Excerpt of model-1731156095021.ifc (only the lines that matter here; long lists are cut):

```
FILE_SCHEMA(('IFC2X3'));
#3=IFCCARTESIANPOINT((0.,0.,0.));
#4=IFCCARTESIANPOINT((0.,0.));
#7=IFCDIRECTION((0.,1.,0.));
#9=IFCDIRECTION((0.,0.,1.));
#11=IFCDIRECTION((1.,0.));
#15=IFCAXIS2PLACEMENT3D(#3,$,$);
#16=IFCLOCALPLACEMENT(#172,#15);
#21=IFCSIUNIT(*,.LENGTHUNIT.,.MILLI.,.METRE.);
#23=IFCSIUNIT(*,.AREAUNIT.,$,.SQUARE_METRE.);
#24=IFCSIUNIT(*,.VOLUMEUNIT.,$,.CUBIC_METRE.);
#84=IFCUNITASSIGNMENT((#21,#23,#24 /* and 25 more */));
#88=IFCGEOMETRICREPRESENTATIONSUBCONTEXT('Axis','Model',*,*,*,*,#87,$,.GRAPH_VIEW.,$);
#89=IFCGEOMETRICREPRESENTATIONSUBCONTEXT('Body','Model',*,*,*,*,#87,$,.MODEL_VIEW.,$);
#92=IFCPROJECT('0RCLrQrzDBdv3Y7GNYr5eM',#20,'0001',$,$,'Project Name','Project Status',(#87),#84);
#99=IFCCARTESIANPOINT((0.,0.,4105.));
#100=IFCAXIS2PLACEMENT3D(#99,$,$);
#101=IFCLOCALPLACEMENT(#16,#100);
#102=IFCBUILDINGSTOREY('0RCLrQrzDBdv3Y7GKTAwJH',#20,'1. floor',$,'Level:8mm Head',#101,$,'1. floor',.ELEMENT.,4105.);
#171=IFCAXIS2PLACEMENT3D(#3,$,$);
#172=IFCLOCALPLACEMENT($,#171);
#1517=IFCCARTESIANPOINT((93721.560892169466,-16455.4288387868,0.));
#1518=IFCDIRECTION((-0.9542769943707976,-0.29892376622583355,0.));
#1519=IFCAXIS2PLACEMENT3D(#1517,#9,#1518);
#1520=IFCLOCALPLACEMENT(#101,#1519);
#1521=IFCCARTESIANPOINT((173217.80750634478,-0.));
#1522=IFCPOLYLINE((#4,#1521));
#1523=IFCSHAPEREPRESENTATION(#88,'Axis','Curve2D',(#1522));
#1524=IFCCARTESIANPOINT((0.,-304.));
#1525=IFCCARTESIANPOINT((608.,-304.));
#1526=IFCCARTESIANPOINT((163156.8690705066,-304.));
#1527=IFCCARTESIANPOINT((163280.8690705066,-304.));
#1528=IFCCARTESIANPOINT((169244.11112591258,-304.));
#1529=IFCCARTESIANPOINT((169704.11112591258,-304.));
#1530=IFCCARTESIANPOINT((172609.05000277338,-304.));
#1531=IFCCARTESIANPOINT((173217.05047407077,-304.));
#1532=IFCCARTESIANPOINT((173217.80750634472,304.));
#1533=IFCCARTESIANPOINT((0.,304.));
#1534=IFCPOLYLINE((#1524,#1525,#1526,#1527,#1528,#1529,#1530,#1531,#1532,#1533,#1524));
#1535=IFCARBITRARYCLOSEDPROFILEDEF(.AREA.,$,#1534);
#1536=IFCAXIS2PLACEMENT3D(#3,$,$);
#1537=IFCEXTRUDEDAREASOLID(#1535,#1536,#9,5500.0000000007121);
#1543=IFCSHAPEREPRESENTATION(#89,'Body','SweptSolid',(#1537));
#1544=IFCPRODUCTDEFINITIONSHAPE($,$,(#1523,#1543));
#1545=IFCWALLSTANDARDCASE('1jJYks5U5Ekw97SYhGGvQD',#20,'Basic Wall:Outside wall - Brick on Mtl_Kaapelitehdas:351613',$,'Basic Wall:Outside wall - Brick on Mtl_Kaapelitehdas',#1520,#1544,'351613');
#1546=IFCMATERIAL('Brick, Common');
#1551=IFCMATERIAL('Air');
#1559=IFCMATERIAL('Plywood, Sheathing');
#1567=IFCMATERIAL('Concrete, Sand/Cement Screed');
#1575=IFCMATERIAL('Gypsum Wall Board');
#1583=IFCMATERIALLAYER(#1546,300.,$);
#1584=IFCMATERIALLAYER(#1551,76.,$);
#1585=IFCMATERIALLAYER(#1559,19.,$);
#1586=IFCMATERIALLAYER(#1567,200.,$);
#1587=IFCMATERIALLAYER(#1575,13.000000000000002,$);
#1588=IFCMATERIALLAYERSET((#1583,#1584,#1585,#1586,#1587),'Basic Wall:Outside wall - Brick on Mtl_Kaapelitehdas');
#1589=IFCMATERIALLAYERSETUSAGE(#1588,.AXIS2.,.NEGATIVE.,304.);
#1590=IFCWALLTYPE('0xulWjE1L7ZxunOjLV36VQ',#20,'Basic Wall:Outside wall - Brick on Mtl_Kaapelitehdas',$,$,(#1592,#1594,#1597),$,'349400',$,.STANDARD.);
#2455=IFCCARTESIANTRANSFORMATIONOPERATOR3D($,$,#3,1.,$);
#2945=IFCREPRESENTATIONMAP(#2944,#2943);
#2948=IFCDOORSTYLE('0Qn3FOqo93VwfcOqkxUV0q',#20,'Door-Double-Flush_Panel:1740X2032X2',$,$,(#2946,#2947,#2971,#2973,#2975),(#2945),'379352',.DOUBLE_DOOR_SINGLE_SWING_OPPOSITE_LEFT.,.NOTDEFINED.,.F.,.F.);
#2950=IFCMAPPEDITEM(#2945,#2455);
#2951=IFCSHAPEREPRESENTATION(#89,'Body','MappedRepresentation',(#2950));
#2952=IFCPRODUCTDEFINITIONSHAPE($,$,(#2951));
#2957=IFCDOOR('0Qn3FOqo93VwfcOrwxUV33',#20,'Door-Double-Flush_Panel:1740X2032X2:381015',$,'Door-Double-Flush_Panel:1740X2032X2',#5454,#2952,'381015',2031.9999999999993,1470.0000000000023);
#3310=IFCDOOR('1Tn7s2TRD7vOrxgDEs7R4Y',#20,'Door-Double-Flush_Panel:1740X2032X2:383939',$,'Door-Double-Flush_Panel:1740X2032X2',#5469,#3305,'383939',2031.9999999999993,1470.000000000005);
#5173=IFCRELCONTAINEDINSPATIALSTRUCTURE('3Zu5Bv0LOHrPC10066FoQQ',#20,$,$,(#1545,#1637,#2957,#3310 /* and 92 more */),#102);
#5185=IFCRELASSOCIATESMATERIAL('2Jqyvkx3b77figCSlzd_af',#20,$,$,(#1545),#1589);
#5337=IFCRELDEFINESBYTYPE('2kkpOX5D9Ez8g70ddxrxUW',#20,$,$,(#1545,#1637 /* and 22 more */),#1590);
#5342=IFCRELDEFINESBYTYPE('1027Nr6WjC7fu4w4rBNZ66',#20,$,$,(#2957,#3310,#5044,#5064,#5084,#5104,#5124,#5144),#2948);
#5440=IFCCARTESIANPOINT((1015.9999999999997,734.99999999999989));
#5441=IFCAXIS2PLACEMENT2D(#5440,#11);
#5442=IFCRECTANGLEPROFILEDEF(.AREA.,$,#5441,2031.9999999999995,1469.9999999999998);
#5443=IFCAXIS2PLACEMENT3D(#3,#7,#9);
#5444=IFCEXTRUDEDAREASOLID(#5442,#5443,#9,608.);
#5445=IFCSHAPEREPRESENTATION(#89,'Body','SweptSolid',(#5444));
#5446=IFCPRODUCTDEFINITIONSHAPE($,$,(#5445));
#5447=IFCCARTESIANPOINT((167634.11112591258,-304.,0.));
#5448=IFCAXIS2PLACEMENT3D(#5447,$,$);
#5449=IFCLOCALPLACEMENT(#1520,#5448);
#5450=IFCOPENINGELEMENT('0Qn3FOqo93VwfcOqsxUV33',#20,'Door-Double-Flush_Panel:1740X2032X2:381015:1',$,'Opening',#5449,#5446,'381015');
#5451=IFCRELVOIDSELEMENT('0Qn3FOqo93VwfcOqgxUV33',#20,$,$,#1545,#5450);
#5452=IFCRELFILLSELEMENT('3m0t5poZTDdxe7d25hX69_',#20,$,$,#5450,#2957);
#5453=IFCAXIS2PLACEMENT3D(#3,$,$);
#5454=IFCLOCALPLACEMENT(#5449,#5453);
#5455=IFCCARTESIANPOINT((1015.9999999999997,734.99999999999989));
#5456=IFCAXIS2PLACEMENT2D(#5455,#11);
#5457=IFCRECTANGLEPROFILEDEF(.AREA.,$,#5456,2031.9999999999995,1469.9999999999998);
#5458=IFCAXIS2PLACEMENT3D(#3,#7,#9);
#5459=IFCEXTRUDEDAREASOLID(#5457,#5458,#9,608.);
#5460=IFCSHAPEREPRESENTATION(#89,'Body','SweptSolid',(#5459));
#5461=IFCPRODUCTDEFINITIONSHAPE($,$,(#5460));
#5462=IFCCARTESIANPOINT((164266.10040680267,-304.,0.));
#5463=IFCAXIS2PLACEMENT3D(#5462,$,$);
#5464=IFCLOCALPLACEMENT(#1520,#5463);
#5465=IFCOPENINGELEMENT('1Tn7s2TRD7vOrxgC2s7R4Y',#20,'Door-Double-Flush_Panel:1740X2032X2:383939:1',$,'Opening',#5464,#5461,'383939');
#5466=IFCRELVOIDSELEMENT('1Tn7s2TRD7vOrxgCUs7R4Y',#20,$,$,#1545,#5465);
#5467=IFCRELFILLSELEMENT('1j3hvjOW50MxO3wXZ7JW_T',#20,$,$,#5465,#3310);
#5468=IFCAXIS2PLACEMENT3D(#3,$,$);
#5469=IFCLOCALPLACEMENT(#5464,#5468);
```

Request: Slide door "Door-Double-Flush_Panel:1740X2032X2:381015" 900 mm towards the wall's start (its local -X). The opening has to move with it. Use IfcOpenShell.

```python
import ifcopenshell
import ifcopenshell.api.geometry
import ifcopenshell.util.placement
import ifcopenshell.util.unit

model = ifcopenshell.open("model-1731156095021.ifc")
unit_scale = ifcopenshell.util.unit.calculate_unit_scale(model)

door = model.by_guid("0Qn3FOqo93VwfcOrwxUV33")
opening = door.FillsVoids[0].RelatingOpeningElement
wall = opening.VoidsElements[0].RelatingBuildingElement

wall_matrix = ifcopenshell.util.placement.get_local_placement(wall.ObjectPlacement)
shift = wall_matrix[:3, 0] * -0.9 / unit_scale
before = ifcopenshell.util.placement.get_local_placement(door.ObjectPlacement)[:3, 3].copy()

# The door is placed relative to its opening, so it follows when the opening moves.
matrix = ifcopenshell.util.placement.get_local_placement(opening.ObjectPlacement)
matrix[:3, 3] += shift
ifcopenshell.api.geometry.edit_object_placement(
    model, product=opening, matrix=matrix, is_si=False, should_transform_children=True
)

after = ifcopenshell.util.placement.get_local_placement(door.ObjectPlacement)[:3, 3]
print("door moved by", (after - before).round(3) + 0.0)

model.write("model-1731156095021_edited.ifc")
```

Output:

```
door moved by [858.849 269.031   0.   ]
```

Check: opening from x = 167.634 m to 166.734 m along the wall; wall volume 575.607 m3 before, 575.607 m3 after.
